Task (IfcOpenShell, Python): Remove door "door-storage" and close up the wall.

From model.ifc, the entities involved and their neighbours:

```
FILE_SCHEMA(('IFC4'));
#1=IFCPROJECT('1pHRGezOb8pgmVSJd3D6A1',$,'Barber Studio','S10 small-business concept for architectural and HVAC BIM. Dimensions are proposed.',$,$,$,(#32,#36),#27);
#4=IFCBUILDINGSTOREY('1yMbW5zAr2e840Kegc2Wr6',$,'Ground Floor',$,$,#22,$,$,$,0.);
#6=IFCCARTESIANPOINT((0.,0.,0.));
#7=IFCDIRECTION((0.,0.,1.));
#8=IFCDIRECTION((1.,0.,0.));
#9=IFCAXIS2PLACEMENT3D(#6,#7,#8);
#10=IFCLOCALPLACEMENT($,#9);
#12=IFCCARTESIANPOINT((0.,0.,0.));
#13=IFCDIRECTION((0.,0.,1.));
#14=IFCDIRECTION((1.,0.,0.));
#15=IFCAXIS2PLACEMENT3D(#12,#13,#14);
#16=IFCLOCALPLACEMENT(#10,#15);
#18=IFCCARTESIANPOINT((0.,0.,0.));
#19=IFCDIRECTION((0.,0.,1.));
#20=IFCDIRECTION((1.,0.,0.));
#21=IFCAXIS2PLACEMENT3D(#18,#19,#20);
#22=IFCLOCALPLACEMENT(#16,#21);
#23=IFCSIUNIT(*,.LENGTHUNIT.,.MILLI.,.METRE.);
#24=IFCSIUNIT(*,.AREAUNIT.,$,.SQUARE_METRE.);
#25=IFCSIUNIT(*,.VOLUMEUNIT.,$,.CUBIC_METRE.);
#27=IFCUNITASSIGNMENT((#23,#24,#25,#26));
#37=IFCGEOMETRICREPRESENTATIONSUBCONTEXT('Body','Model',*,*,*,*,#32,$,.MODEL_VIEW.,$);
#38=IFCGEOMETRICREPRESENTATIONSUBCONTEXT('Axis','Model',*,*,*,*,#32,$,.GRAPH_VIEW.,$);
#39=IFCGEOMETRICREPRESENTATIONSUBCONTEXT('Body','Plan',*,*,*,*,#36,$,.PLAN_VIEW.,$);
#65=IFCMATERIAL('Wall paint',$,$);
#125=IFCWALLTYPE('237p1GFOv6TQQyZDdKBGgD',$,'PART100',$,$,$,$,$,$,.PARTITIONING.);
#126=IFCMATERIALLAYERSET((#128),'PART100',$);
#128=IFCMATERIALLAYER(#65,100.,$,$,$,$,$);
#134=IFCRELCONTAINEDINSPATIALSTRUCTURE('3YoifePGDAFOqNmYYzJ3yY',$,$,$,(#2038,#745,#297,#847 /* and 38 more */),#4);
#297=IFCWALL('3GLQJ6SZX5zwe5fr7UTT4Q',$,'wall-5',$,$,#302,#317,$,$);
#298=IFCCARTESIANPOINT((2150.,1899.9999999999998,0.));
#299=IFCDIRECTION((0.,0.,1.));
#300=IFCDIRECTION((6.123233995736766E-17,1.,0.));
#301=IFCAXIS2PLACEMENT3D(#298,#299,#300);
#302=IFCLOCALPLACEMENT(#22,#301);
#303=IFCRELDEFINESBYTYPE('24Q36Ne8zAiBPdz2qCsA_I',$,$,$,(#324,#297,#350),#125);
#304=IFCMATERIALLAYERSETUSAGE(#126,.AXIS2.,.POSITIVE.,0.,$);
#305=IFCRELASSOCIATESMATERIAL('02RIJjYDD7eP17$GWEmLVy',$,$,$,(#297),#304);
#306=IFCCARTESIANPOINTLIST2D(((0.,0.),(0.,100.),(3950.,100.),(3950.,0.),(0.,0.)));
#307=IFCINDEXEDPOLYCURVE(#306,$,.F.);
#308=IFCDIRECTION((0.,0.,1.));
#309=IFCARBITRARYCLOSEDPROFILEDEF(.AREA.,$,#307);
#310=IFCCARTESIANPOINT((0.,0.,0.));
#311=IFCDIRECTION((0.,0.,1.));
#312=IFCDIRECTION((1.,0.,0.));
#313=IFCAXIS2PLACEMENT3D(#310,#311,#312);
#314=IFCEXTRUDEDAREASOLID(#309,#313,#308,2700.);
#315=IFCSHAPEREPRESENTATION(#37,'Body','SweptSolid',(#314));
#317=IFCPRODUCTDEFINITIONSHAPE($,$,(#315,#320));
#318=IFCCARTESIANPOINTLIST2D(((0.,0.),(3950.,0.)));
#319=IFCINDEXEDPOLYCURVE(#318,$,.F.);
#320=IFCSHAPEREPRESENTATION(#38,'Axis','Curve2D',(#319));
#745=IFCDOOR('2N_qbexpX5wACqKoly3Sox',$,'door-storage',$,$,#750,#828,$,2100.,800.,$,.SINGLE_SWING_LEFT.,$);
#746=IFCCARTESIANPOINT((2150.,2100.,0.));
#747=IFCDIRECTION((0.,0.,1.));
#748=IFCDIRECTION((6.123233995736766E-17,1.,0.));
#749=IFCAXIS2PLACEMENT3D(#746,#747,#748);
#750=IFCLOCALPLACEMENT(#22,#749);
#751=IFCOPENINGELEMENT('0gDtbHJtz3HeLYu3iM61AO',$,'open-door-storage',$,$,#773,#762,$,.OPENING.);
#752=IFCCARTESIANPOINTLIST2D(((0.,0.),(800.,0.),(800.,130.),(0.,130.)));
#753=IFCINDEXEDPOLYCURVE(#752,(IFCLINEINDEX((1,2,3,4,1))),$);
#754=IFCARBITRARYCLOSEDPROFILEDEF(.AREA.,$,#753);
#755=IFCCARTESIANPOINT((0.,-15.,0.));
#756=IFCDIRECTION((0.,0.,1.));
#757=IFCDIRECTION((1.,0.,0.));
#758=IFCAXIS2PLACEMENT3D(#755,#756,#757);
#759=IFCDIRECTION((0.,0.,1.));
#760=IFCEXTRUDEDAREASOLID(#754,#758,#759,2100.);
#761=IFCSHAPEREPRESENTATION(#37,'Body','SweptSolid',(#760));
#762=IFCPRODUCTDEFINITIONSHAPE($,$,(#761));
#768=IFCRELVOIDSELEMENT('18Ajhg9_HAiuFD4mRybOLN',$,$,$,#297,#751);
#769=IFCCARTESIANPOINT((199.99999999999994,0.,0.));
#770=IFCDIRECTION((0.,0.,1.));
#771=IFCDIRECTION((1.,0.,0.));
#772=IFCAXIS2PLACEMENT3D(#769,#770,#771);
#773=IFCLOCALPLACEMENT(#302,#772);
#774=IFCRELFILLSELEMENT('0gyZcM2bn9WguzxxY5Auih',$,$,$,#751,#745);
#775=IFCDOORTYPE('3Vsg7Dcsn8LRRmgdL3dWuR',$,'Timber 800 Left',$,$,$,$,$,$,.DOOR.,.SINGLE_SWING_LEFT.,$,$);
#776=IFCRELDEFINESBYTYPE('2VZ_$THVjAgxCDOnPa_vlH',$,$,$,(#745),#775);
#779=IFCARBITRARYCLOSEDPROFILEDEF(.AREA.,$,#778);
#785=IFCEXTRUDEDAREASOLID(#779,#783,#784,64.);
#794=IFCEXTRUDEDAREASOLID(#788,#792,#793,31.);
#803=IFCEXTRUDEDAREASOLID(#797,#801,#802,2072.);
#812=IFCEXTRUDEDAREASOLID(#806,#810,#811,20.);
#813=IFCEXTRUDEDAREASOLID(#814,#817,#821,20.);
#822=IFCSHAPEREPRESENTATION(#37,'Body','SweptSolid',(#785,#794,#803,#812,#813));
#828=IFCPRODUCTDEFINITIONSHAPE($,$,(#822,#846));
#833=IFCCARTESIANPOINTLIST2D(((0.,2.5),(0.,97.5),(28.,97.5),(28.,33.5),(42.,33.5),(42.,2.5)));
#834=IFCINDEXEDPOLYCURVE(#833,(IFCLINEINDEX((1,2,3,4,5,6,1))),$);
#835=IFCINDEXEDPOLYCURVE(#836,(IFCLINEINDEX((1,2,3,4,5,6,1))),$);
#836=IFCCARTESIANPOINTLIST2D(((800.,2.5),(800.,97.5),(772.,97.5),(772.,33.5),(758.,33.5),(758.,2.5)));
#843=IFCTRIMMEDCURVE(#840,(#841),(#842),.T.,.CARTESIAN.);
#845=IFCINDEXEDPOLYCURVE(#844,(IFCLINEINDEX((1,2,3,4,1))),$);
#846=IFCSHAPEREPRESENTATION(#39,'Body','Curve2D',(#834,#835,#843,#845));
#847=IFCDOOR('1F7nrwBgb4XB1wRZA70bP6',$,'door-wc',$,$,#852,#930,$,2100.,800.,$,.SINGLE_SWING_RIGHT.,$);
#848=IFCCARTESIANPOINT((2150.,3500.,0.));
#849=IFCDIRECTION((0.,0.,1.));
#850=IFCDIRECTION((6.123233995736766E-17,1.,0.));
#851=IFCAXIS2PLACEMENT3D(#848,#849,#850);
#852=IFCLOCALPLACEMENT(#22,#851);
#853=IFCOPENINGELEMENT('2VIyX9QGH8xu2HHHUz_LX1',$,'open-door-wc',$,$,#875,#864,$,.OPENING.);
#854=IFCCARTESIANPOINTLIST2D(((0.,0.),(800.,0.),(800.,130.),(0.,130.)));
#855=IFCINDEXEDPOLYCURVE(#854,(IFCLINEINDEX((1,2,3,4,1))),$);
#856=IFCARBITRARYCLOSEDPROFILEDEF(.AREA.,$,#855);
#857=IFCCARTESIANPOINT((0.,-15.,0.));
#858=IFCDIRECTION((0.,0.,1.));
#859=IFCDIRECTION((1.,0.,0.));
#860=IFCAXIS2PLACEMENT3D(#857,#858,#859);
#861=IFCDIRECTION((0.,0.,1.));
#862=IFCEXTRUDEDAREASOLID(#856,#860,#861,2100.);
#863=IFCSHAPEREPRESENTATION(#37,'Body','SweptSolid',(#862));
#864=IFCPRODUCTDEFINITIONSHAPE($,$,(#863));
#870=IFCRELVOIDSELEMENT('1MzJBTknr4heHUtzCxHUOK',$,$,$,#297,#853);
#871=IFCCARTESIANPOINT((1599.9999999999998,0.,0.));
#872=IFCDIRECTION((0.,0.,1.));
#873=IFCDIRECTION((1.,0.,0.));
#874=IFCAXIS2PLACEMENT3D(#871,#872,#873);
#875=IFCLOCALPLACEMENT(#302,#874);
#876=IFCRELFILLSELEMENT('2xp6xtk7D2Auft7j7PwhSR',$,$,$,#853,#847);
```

```python
import ifcopenshell
import ifcopenshell.api.feature
import ifcopenshell.api.root
import ifcopenshell.geom
import ifcopenshell.util.shape

model = ifcopenshell.open("model.ifc")
settings = ifcopenshell.geom.settings()


def volume(element):
    """Net volume in cubic metres, openings subtracted."""
    shape = ifcopenshell.geom.create_shape(settings, element)
    return ifcopenshell.util.shape.get_volume(shape.geometry)


door = model.by_guid("2N_qbexpX5wACqKoly3Sox")
opening = door.FillsVoids[0].RelatingOpeningElement
wall = opening.VoidsElements[0].RelatingBuildingElement
before = volume(wall)

ifcopenshell.api.root.remove_product(model, product=door)
ifcopenshell.api.feature.remove_feature(model, feature=opening)

after = volume(wall)

print(f"wall volume {before:.3f} -> {after:.3f} m3")

model.write("model_edited.ifc")
```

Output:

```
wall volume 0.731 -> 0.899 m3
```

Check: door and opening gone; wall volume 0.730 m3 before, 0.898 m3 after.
